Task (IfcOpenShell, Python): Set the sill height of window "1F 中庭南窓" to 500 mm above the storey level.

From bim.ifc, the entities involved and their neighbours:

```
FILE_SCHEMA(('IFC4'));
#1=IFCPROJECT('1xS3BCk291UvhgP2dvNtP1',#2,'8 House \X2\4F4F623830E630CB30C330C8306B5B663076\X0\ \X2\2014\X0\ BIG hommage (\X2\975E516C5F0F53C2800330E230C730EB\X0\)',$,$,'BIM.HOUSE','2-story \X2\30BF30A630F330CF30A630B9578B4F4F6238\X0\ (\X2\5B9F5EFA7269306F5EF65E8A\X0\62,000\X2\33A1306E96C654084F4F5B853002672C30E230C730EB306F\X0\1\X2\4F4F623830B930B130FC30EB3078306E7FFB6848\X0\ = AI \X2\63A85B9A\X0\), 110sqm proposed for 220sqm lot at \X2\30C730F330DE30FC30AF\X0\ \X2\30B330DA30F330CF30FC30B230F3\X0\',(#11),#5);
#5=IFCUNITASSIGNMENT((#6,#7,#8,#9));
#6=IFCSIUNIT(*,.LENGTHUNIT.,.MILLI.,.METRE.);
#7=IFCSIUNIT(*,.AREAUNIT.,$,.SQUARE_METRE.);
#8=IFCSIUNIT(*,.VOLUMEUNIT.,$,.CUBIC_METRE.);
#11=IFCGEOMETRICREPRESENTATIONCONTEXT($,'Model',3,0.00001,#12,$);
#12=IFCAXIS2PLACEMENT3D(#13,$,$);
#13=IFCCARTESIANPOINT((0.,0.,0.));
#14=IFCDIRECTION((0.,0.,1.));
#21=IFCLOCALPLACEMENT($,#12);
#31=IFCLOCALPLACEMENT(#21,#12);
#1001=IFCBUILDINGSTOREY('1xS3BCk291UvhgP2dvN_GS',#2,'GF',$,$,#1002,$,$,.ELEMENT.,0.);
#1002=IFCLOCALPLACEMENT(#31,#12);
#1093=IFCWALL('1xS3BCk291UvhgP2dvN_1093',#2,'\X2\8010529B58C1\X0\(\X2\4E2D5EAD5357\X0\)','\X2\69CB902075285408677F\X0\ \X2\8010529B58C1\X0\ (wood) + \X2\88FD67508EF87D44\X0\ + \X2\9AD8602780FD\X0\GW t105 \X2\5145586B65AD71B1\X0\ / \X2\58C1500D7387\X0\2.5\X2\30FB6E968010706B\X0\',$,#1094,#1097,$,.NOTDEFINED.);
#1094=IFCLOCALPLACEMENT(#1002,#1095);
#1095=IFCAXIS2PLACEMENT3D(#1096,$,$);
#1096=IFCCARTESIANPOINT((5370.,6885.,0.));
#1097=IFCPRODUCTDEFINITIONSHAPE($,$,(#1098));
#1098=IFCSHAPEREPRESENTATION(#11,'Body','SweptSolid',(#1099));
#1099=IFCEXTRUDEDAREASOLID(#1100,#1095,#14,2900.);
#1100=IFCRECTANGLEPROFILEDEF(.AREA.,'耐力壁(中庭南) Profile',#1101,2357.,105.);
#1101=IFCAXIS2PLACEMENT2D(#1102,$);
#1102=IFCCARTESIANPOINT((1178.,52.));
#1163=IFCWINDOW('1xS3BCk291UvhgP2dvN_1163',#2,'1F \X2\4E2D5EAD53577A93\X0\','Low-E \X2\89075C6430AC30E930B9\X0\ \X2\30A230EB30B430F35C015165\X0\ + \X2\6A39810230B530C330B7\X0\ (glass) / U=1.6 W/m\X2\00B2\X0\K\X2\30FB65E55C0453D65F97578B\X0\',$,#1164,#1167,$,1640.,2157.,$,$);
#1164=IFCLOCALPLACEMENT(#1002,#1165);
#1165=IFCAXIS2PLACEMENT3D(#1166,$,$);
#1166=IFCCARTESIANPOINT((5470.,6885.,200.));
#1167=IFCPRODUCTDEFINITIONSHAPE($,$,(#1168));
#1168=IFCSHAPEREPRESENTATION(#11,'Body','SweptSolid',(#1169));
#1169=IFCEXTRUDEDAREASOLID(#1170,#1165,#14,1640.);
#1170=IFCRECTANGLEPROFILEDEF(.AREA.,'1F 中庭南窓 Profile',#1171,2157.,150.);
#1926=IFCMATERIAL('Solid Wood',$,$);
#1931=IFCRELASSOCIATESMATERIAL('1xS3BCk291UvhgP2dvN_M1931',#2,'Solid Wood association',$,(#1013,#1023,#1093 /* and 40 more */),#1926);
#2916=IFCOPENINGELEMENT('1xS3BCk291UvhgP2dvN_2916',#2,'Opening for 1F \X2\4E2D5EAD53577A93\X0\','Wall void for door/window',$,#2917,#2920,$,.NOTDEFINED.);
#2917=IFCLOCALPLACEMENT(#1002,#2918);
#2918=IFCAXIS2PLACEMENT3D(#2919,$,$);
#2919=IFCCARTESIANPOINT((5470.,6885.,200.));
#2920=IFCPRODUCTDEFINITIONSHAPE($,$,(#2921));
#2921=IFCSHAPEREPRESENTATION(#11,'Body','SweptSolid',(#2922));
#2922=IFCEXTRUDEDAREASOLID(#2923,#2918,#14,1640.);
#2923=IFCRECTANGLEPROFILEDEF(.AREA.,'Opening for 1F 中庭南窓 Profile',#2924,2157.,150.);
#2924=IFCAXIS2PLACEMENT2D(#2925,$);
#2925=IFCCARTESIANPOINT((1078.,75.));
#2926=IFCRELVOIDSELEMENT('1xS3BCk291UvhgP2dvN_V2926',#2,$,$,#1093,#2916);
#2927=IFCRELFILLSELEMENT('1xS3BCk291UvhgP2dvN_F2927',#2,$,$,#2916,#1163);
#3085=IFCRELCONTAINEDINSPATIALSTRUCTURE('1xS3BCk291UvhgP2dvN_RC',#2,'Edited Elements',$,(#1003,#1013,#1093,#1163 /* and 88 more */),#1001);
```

```python
import numpy as np
import ifcopenshell
import ifcopenshell.api.geometry
import ifcopenshell.geom
import ifcopenshell.util.element
import ifcopenshell.util.placement
import ifcopenshell.util.shape
import ifcopenshell.util.unit

model = ifcopenshell.open("bim.ifc")
unit_scale = ifcopenshell.util.unit.calculate_unit_scale(model)

window = model.by_guid("1xS3BCk291UvhgP2dvN_1163")
opening = window.FillsVoids[0].RelatingOpeningElement
storey = ifcopenshell.util.element.get_container(window, ifc_class="IfcBuildingStorey")
level = ifcopenshell.util.placement.get_local_placement(storey.ObjectPlacement)[2, 3]

# The opening's origin need not be at the sill, so measure its lowest point.
shape = ifcopenshell.geom.create_shape(ifcopenshell.geom.settings(), opening)
bottom = ifcopenshell.util.shape.get_shape_bottom_elevation(shape, shape.geometry) / unit_scale
dz = level + 500.0 - bottom

shift = np.array([0.0, 0.0, dz])
# The window is not placed relative to its opening, so move both.
for product in (opening, window):
    matrix = ifcopenshell.util.placement.get_local_placement(product.ObjectPlacement)
    matrix[:3, 3] += shift
    ifcopenshell.api.geometry.edit_object_placement(model, product=product, matrix=matrix, is_si=False)

print(f"moved by {dz * unit_scale:+.3f} m")

model.write("bim_rev.ifc")
```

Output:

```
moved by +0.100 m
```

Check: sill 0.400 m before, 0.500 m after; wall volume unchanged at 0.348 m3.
